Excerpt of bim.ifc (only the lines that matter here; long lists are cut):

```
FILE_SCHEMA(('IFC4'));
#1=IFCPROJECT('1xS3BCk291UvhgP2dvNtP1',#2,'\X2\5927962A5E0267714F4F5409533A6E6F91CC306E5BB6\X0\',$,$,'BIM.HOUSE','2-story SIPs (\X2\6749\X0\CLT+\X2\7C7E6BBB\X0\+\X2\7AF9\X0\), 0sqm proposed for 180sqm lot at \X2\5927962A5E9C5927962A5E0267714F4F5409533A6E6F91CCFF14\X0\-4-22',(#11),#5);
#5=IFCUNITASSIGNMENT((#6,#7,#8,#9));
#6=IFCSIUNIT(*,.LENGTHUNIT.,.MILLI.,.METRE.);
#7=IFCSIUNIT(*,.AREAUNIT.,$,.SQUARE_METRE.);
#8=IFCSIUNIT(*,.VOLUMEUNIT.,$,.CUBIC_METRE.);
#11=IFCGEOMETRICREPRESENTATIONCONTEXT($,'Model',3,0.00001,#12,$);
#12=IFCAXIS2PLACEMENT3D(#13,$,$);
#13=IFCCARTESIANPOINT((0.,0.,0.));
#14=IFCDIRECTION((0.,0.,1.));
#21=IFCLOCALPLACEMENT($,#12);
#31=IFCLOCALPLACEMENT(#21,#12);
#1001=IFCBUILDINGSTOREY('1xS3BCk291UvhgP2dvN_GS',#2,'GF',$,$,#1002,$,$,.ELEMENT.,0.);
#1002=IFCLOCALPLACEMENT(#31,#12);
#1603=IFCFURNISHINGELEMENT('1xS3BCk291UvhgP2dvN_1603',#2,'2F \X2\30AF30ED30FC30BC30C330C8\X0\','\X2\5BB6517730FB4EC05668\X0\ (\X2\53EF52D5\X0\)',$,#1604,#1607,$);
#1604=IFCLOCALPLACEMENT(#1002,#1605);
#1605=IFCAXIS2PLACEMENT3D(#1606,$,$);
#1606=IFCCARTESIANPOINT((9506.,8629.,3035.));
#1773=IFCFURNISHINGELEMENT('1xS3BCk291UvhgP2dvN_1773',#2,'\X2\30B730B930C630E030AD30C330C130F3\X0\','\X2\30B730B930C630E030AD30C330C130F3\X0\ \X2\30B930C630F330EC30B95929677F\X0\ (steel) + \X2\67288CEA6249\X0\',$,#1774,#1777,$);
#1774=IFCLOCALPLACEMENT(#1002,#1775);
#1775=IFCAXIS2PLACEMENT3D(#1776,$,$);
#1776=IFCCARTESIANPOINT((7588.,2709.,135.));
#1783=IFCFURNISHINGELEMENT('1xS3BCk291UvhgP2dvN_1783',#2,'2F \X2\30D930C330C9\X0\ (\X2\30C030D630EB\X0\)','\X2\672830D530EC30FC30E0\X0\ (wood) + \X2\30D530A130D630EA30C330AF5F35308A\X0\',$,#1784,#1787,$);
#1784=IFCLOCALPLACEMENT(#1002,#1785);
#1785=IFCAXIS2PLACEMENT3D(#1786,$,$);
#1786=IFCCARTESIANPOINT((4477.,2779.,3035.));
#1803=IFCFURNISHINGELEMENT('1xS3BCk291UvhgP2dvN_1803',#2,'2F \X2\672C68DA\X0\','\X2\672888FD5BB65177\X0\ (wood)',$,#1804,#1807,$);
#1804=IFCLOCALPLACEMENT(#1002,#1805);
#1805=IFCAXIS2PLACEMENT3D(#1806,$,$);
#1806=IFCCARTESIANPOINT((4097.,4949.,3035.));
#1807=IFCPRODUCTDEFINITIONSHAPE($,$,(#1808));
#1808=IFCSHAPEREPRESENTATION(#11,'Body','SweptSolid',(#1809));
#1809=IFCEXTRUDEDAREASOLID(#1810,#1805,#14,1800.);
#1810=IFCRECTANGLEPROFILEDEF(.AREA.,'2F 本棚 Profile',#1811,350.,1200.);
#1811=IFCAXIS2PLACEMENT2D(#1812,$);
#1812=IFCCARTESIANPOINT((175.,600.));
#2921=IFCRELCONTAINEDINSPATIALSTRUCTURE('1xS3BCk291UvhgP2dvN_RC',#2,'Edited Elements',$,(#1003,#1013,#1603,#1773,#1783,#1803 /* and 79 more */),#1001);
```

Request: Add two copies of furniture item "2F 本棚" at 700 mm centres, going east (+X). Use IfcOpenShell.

```python
import numpy as np
import ifcopenshell
import ifcopenshell.api.geometry
import ifcopenshell.api.root
import ifcopenshell.util.element
import ifcopenshell.util.placement
import ifcopenshell.util.unit

model = ifcopenshell.open("bim.ifc")
unit_scale = ifcopenshell.util.unit.calculate_unit_scale(model)


def reuse_history(source, copy):
    """copy_class also copies each property set's owner history, people and application; keep the originals."""
    for rel in copy.IsDefinedBy:
        if rel.is_a("IfcRelDefinesByProperties") and (history := rel.RelatingPropertyDefinition.OwnerHistory):
            rel.RelatingPropertyDefinition.OwnerHistory = source.OwnerHistory
            ifcopenshell.util.element.remove_deep2(model, history)


source = model.by_id(1803)
base = ifcopenshell.util.placement.get_local_placement(source.ObjectPlacement)
step = np.array([1.0, 0.0, 0.0]) * 0.7 / unit_scale

for i in range(1, 3):
    copy = ifcopenshell.api.root.copy_class(model, product=source)
    copy.Representation = ifcopenshell.util.element.copy_deep(
        model, source.Representation, exclude=["IfcGeometricRepresentationContext", "IfcRepresentationMap"]
    )
    reuse_history(source, copy)
    matrix = base.copy()
    matrix[:3, 3] += i * step
    print("added at", matrix[:3, 3].round(3) + 0.0)
    ifcopenshell.api.geometry.edit_object_placement(model, product=copy, matrix=matrix, is_si=False)

model.write("bim_edited.ifc")
```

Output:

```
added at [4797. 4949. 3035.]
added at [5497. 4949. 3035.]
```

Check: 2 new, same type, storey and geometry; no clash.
